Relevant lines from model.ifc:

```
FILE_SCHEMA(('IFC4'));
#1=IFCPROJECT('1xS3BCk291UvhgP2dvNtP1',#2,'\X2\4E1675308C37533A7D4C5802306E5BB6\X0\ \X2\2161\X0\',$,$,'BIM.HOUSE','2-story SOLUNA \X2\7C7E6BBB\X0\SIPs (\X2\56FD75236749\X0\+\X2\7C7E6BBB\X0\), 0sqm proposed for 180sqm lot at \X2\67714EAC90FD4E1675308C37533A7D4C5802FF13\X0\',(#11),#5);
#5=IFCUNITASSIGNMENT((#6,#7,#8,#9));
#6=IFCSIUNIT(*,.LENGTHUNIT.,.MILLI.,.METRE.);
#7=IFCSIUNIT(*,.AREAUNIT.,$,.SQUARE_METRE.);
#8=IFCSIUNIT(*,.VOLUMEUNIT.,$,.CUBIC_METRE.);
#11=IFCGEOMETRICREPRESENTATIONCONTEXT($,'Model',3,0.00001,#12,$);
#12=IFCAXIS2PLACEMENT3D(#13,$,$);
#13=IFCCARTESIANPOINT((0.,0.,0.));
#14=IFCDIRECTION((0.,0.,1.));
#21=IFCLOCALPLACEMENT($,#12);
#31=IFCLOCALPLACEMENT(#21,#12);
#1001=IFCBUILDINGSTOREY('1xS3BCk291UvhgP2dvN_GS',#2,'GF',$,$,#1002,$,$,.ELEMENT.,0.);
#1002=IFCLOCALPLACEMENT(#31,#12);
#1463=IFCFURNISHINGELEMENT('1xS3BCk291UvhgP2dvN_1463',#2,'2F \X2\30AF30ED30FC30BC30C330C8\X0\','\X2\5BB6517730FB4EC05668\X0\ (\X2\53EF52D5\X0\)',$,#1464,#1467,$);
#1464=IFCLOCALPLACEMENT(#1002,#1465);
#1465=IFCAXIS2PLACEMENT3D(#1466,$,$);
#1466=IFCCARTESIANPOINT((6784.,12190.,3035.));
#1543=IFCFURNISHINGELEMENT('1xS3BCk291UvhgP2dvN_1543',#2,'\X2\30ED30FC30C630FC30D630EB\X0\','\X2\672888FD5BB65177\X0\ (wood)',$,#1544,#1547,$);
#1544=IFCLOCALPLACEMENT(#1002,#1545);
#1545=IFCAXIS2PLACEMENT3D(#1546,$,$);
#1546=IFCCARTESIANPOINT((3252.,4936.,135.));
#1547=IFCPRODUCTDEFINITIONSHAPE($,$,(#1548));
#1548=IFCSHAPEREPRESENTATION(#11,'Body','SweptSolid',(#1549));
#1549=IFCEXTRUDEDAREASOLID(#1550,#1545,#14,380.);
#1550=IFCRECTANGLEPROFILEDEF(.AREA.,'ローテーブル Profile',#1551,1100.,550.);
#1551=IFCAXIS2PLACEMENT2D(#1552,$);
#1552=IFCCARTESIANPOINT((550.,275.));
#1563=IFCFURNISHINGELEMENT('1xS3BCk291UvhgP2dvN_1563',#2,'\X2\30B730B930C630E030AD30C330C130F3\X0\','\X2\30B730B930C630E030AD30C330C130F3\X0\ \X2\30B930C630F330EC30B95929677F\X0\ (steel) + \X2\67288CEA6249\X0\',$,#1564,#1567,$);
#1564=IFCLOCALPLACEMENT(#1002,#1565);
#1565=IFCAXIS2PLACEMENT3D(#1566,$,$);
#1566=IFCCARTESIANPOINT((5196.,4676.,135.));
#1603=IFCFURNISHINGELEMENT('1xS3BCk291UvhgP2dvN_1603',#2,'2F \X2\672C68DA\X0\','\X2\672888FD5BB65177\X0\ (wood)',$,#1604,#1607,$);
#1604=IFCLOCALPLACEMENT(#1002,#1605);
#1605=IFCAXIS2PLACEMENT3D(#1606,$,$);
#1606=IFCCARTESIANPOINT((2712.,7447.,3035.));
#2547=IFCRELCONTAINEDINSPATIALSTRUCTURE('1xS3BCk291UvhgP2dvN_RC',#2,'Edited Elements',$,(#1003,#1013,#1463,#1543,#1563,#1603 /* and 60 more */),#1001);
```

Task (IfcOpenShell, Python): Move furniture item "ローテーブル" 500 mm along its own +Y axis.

```python
import ifcopenshell
import ifcopenshell.api.geometry
import ifcopenshell.util.placement

model = ifcopenshell.open("model.ifc")

item = model.by_id(1543)
matrix = ifcopenshell.util.placement.get_local_placement(item.ObjectPlacement)
matrix[:3, 3] += matrix[:3, 1] * 500.0
ifcopenshell.api.geometry.edit_object_placement(model, product=item, matrix=matrix, is_si=False)

print(ifcopenshell.util.placement.get_local_placement(item.ObjectPlacement).round(3) + 0.0)

model.write("model_updated.ifc")
```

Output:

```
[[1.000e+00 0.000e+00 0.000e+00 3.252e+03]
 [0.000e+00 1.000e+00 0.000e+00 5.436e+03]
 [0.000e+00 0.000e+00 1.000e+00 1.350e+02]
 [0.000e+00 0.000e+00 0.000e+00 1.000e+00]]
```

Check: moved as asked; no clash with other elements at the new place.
